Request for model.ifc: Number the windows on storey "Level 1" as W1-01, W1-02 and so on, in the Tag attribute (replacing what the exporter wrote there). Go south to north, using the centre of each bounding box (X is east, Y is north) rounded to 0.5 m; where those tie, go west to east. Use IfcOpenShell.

First a look at what the model holds.

```python
import ifcopenshell
import ifcopenshell.util.element
import ifcopenshell.util.placement

model = ifcopenshell.open("model.ifc")
print(model.schema)
storey = next(s for s in model.by_type("IfcBuildingStorey") if s.Name == "Level 1")
windows = [e for e in ifcopenshell.util.element.get_decomposition(storey) if e.is_a("IfcWindow")]
for e in sorted(windows, key=lambda e: e.id()):
    origin = ifcopenshell.util.placement.get_local_placement(e.ObjectPlacement)[:3, 3]
    print(e.id(), e.Tag, e.Name, origin.round(2) + 0.0, sep=" | ")
```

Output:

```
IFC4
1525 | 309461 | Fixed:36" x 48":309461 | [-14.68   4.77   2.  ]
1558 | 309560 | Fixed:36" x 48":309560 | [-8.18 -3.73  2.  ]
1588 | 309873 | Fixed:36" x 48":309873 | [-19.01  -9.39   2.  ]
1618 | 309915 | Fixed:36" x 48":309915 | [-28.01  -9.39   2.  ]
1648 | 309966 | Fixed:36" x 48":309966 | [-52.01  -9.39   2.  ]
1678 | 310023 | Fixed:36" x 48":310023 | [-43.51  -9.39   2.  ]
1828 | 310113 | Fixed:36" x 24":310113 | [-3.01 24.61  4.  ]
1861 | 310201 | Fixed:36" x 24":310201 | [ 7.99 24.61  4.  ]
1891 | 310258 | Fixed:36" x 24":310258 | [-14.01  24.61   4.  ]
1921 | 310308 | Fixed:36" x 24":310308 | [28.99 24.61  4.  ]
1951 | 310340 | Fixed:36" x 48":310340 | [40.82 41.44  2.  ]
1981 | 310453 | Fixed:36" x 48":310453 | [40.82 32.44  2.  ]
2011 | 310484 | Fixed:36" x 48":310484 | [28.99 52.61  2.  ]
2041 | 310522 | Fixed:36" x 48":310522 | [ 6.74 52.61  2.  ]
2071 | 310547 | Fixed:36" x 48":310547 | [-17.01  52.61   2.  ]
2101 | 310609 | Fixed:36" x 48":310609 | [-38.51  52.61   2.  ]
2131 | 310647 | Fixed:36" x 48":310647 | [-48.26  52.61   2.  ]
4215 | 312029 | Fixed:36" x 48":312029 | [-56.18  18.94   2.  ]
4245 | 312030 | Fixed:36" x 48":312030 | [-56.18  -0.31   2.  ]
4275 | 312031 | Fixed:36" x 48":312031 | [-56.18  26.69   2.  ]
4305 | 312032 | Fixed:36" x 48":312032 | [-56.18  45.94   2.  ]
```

```python
import ifcopenshell
import ifcopenshell.geom
import ifcopenshell.util.element
import ifcopenshell.util.shape

model = ifcopenshell.open("model.ifc")
settings = ifcopenshell.geom.settings()
settings.set("use-world-coords", True)


def centre(element):
    shape = ifcopenshell.geom.create_shape(settings, element)
    return ifcopenshell.util.shape.get_bbox_centroid(shape.geometry)


storey = next(s for s in model.by_type("IfcBuildingStorey") if s.Name == "Level 1")
windows = [e for e in ifcopenshell.util.element.get_decomposition(storey) if e.is_a("IfcWindow")]

# Insertion points can sit at a corner or the storey origin, so sort by the geometry (in metres).
centres = {e: centre(e) for e in windows}
windows.sort(key=lambda e: (round(centres[e][1] / 0.5), centres[e][0]))

for i, e in enumerate(windows, start=1):
    number = f"W1-{i:02d}"
    e.Tag = number
    print(e.id(), number)

model.write("model_rev.ifc")
```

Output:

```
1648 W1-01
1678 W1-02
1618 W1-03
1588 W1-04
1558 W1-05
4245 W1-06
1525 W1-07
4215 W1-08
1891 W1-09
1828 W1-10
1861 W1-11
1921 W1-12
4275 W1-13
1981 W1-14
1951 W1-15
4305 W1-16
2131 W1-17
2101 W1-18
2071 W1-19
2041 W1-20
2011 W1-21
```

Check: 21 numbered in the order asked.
